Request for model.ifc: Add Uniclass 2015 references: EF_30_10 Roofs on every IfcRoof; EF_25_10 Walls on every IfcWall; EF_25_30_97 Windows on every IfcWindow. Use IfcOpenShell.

First a look at what the model holds.

```python
import ifcopenshell

model = ifcopenshell.open("model.ifc")
print(model.schema)
print("classifications:", [c.Name for c in model.by_type("IfcClassification")])
for ifc_class in ("IfcDoor", "IfcRoof", "IfcStair", "IfcWall", "IfcWindow"):
    print(ifc_class, len(model.by_type(ifc_class)))
```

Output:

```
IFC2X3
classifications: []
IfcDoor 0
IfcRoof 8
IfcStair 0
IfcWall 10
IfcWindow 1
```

```python
import ifcopenshell
import ifcopenshell.api.classification

model = ifcopenshell.open("model.ifc")

# IFC2X3 requires Source and Edition and has no link from the project to the system.
system = model.create_entity("IfcClassification", Source="NBS", Edition="2015", Name="Uniclass 2015")

codes = {
    "IfcRoof": ("EF_30_10", "Roofs"),
    "IfcWall": ("EF_25_10", "Walls"),
    "IfcWindow": ("EF_25_30_97", "Windows"),
}
for ifc_class, (code, name) in codes.items():
    products = model.by_type(ifc_class)
    ifcopenshell.api.classification.add_reference(
        model, products=products, classification=system, identification=code, name=name
    )
    print(code, len(products))

model.write("model_v2.ifc")
```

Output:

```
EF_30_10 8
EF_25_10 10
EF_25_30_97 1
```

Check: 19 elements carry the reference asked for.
